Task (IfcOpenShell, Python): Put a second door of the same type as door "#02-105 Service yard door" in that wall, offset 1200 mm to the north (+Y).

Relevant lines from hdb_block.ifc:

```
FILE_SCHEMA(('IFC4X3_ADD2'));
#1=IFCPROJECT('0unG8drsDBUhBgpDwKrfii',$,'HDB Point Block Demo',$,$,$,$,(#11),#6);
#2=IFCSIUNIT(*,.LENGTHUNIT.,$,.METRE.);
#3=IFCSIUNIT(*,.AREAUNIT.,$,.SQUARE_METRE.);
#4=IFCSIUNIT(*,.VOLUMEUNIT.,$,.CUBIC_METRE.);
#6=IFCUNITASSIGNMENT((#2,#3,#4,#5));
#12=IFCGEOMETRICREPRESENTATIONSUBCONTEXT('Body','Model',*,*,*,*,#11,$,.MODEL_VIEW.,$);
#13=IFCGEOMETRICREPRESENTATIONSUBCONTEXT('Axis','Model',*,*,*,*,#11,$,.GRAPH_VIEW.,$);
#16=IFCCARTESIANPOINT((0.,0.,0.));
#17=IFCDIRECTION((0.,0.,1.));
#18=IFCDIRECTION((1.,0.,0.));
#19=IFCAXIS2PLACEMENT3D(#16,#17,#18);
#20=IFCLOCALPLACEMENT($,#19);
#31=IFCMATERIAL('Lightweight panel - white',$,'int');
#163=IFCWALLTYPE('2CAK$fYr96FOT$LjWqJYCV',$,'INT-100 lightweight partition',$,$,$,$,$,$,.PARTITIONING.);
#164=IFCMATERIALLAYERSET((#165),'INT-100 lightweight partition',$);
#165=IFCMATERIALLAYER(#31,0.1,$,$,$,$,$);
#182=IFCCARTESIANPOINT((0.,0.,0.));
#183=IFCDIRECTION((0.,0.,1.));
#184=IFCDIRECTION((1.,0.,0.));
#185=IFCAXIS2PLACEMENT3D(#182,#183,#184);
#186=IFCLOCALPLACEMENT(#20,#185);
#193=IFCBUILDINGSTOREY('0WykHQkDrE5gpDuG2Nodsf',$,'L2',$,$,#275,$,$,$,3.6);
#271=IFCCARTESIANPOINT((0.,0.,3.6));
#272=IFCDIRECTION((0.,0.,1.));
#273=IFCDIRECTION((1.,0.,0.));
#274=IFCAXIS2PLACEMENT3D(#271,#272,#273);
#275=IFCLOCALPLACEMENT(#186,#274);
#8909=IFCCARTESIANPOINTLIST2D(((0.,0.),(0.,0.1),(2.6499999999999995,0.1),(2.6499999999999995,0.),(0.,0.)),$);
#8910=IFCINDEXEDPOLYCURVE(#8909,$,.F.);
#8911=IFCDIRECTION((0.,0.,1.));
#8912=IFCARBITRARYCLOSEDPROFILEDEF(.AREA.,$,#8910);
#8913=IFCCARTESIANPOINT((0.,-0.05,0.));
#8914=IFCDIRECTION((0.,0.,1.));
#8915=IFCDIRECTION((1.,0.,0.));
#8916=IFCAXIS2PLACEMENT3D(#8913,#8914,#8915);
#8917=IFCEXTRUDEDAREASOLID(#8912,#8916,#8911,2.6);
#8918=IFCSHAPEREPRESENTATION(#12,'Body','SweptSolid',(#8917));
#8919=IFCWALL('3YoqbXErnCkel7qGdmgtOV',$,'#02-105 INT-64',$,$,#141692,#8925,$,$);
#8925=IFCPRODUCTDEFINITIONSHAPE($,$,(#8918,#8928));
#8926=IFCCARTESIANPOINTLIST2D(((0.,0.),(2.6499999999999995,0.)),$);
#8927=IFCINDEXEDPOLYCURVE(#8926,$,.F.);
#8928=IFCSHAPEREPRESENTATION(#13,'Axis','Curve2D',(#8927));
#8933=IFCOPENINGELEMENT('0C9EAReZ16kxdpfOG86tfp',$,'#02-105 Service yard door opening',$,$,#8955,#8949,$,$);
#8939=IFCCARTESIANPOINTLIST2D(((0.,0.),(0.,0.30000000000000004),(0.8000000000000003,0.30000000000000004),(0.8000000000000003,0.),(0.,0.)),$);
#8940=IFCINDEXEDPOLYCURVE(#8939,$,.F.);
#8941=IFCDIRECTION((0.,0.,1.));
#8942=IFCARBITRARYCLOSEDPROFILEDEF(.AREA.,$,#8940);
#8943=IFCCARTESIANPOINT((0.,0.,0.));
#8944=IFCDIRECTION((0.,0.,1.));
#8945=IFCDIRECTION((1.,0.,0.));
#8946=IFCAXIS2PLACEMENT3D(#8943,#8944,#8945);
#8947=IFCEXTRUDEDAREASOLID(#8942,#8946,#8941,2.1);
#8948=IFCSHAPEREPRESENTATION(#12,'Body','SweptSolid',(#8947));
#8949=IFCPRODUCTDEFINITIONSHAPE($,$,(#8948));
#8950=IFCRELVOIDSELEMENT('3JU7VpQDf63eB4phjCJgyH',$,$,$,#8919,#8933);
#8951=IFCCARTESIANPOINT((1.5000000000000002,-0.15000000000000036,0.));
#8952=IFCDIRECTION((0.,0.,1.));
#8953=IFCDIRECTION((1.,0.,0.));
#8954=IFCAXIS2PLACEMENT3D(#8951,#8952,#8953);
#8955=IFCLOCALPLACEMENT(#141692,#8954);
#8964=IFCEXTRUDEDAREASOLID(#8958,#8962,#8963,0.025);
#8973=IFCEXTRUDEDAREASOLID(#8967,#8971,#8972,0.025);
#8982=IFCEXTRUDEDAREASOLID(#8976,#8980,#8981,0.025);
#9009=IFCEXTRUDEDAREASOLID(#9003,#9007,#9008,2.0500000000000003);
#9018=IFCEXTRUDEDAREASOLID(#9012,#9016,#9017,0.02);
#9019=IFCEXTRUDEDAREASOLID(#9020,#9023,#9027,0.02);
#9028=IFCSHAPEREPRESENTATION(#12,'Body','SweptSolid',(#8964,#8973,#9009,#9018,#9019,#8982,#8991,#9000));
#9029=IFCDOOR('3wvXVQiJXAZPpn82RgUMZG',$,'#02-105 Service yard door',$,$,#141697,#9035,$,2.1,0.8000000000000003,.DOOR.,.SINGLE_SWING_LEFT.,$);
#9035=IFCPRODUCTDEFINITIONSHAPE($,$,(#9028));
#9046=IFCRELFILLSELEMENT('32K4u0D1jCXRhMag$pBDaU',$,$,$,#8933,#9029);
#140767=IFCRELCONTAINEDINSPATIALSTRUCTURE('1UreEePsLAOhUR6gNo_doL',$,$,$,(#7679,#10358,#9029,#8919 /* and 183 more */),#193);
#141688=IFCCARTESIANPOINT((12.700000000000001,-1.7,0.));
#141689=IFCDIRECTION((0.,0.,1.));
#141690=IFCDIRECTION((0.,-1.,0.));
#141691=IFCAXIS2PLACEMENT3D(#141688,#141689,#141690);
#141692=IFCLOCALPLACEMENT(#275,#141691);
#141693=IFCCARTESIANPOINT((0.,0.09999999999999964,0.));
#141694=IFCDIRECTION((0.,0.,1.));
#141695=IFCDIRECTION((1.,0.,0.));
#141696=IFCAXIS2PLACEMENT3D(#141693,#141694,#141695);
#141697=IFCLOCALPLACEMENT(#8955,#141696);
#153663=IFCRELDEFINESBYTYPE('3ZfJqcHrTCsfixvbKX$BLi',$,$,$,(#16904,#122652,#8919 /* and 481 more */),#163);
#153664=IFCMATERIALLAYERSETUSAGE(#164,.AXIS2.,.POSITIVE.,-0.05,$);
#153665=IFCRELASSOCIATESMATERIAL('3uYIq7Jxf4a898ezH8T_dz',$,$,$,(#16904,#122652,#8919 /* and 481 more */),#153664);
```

```python
import ifcopenshell
import ifcopenshell.api.feature
import ifcopenshell.api.geometry
import ifcopenshell.api.root
import ifcopenshell.geom
import ifcopenshell.util.element
import ifcopenshell.util.placement
import ifcopenshell.util.shape
import ifcopenshell.util.unit

model = ifcopenshell.open("hdb_block.ifc")
unit_scale = ifcopenshell.util.unit.calculate_unit_scale(model)
settings = ifcopenshell.geom.settings()


def volume(element):
    """Net volume in cubic metres, openings subtracted."""
    shape = ifcopenshell.geom.create_shape(settings, element)
    return ifcopenshell.util.shape.get_volume(shape.geometry)


door = model.by_guid("3wvXVQiJXAZPpn82RgUMZG")
opening = door.FillsVoids[0].RelatingOpeningElement
wall = opening.VoidsElements[0].RelatingBuildingElement
before = volume(wall)
shift = ifcopenshell.util.placement.get_local_placement(wall.ObjectPlacement)[:3, 0] * -1.2 / unit_scale

# copy_class copies the void relationship, type, container and properties, but no geometry.
new_opening = ifcopenshell.api.root.copy_class(model, product=opening)
new_opening.Representation = ifcopenshell.util.element.copy_deep(
    model, opening.Representation, exclude=["IfcGeometricRepresentationContext", "IfcRepresentationMap"]
)
new_door = ifcopenshell.api.root.copy_class(model, product=door)
new_door.Representation = ifcopenshell.util.element.copy_deep(
    model, door.Representation, exclude=["IfcGeometricRepresentationContext", "IfcRepresentationMap"]
)
ifcopenshell.api.feature.add_filling(model, opening=new_opening, element=new_door)

for old, new in ((opening, new_opening), (door, new_door)):
    matrix = ifcopenshell.util.placement.get_local_placement(old.ObjectPlacement)
    matrix[:3, 3] += shift
    ifcopenshell.api.geometry.edit_object_placement(model, product=new, matrix=matrix, is_si=False)

after = volume(wall)

print(f"wall volume {before:.3f} -> {after:.3f} m3")

model.write("hdb_block_updated.ifc")
```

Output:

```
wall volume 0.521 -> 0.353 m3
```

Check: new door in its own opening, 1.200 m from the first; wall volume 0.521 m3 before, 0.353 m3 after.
